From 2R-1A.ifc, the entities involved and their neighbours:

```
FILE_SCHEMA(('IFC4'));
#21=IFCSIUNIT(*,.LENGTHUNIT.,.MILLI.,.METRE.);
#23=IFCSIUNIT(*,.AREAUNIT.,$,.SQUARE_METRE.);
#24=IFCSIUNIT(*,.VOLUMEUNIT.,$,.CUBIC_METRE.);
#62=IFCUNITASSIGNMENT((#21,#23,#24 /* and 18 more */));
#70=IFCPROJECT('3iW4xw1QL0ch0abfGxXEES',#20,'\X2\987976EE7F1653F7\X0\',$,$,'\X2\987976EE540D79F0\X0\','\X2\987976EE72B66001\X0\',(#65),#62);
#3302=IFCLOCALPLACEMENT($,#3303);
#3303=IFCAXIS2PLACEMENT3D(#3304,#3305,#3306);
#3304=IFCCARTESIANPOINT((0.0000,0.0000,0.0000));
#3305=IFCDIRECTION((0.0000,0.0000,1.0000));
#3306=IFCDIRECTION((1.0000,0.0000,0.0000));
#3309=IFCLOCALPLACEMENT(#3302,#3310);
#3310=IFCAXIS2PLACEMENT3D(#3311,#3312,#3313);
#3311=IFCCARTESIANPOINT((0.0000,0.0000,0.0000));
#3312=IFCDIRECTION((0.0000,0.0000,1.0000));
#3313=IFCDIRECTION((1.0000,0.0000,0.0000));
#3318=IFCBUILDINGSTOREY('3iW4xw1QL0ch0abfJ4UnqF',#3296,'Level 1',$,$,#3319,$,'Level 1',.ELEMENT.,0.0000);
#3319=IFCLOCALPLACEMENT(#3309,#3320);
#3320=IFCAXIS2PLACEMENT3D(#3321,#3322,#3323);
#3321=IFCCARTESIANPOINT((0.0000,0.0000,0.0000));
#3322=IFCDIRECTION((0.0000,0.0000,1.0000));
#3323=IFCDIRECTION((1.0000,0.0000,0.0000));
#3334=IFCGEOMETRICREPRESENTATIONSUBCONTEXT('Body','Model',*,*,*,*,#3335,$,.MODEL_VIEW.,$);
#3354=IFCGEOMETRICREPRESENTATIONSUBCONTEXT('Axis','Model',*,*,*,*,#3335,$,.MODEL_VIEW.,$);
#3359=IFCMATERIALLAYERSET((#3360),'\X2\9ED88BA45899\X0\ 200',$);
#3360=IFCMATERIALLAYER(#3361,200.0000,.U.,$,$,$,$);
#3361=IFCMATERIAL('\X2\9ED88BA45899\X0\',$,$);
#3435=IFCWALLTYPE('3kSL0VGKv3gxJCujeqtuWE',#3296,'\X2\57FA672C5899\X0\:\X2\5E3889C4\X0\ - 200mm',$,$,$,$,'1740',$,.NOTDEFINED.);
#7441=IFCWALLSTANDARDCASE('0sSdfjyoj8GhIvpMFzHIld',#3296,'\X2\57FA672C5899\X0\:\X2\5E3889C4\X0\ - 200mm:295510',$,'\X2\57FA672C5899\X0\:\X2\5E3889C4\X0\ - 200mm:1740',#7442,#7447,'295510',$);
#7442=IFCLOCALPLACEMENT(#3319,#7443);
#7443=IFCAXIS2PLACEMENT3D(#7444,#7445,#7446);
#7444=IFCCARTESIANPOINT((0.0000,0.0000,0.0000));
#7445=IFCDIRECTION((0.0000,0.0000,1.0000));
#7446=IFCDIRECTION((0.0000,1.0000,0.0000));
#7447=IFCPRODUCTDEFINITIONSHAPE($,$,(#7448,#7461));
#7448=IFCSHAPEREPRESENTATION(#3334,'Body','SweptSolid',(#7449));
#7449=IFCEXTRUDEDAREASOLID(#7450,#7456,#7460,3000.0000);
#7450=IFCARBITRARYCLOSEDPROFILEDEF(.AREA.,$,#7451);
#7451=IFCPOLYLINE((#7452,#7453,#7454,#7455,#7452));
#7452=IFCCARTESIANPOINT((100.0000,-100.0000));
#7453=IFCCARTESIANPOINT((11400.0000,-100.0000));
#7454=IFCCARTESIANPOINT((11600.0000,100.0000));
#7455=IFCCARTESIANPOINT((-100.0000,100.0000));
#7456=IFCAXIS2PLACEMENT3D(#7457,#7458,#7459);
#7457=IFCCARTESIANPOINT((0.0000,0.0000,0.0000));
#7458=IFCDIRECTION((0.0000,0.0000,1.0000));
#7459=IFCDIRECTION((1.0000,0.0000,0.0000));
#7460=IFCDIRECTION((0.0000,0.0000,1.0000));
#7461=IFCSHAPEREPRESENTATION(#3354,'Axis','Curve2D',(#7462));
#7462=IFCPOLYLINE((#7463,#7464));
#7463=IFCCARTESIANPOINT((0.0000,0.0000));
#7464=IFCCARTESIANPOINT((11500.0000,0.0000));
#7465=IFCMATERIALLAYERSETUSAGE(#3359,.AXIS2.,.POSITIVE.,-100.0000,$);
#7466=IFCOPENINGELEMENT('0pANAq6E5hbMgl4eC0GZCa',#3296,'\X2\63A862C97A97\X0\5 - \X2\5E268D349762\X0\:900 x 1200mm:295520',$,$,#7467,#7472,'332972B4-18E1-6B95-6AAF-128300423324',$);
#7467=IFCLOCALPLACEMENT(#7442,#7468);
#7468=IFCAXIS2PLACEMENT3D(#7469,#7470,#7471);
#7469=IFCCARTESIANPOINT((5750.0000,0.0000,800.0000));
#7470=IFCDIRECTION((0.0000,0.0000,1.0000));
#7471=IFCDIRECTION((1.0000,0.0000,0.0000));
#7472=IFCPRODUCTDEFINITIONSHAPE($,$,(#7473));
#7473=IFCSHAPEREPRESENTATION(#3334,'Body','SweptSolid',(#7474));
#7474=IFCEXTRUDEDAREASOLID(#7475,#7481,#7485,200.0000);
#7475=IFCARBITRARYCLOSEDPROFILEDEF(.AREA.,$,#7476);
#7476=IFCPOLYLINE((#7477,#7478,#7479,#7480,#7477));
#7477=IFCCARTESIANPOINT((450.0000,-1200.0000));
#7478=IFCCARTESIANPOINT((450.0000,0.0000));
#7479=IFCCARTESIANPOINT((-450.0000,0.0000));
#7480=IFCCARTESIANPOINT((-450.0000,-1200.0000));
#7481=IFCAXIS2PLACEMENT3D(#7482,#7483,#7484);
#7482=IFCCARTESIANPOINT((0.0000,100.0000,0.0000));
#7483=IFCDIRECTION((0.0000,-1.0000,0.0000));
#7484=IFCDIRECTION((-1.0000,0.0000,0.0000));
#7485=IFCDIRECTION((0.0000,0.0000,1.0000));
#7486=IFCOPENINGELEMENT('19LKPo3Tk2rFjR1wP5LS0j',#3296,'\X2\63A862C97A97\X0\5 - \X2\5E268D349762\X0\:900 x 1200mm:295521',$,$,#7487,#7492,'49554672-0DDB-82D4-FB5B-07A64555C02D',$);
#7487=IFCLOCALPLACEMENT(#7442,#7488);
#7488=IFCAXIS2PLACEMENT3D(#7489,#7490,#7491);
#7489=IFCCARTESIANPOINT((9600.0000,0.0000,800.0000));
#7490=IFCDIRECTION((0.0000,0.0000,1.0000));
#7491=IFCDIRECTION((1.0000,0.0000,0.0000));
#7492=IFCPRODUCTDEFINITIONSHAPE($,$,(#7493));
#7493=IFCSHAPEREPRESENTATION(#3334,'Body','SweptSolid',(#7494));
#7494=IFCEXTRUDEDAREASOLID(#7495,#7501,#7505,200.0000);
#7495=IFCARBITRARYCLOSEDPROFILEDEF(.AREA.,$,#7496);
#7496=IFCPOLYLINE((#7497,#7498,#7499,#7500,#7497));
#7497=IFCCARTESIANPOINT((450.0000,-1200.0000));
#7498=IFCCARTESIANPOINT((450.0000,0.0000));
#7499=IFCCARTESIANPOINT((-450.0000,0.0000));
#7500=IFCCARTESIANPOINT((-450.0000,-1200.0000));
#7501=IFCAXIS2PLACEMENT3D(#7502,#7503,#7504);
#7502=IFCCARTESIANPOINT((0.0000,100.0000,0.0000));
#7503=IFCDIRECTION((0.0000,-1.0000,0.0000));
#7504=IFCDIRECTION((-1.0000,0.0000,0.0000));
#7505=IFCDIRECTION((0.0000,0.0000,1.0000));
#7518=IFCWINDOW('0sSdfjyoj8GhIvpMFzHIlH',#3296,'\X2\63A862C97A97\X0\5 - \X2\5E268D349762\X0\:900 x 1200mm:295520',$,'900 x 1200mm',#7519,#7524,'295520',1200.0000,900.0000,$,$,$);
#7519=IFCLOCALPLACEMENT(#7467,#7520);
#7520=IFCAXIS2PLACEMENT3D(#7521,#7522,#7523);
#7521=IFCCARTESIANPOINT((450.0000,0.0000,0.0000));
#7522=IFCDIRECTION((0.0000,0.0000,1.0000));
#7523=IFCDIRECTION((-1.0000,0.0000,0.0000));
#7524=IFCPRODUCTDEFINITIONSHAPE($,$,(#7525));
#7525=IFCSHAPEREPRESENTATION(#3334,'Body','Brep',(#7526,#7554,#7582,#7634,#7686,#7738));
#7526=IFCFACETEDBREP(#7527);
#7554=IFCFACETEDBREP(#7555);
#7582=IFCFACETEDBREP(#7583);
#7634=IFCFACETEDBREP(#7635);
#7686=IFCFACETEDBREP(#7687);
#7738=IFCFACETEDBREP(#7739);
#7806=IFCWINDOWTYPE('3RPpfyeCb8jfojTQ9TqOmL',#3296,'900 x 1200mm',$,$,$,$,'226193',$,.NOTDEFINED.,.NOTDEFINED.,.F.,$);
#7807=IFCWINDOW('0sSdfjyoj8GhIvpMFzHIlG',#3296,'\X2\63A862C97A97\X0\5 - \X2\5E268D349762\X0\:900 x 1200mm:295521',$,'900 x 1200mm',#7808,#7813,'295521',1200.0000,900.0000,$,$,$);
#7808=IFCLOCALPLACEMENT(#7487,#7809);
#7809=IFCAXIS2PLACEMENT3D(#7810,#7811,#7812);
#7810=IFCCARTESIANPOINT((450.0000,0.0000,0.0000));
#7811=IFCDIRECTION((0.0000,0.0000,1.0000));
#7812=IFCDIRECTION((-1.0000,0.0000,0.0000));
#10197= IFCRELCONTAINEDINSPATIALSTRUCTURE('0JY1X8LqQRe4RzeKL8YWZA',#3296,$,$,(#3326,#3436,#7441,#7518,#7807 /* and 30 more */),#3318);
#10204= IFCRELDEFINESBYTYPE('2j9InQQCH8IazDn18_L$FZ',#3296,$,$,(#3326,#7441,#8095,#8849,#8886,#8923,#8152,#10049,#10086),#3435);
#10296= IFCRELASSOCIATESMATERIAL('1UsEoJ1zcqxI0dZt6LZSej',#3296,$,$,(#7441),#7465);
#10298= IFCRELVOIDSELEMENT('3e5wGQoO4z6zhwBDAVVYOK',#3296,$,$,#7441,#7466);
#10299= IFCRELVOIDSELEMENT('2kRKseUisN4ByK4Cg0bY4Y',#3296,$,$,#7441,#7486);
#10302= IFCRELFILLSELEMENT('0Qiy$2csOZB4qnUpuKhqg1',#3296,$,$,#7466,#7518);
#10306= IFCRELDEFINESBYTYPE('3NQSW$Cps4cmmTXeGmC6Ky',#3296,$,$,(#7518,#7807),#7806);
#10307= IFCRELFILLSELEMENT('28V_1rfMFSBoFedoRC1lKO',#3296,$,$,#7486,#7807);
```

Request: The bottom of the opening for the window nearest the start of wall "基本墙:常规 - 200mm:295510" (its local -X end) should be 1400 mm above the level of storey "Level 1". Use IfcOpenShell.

```python
import numpy as np
import ifcopenshell
import ifcopenshell.api.geometry
import ifcopenshell.geom
import ifcopenshell.util.element
import ifcopenshell.util.placement
import ifcopenshell.util.shape
import ifcopenshell.util.unit

model = ifcopenshell.open("2R-1A.ifc")
unit_scale = ifcopenshell.util.unit.calculate_unit_scale(model)

window = model.by_id(7518)
opening = window.FillsVoids[0].RelatingOpeningElement
storey = ifcopenshell.util.element.get_container(window, ifc_class="IfcBuildingStorey")
level = ifcopenshell.util.placement.get_local_placement(storey.ObjectPlacement)[2, 3]

# The opening's origin need not be at the sill, so measure its lowest point.
shape = ifcopenshell.geom.create_shape(ifcopenshell.geom.settings(), opening)
bottom = ifcopenshell.util.shape.get_shape_bottom_elevation(shape, shape.geometry) / unit_scale
dz = level + 1.4 / unit_scale - bottom

shift = np.array([0.0, 0.0, dz])
# The window is placed relative to its opening, so it follows when the opening moves.
matrix = ifcopenshell.util.placement.get_local_placement(opening.ObjectPlacement)
matrix[:3, 3] += shift
ifcopenshell.api.geometry.edit_object_placement(
    model, product=opening, matrix=matrix, is_si=False, should_transform_children=True
)

print(f"moved by {dz * unit_scale:+.3f} m")

model.write("2R-1A_edited.ifc")
```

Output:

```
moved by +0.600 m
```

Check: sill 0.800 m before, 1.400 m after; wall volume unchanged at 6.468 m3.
